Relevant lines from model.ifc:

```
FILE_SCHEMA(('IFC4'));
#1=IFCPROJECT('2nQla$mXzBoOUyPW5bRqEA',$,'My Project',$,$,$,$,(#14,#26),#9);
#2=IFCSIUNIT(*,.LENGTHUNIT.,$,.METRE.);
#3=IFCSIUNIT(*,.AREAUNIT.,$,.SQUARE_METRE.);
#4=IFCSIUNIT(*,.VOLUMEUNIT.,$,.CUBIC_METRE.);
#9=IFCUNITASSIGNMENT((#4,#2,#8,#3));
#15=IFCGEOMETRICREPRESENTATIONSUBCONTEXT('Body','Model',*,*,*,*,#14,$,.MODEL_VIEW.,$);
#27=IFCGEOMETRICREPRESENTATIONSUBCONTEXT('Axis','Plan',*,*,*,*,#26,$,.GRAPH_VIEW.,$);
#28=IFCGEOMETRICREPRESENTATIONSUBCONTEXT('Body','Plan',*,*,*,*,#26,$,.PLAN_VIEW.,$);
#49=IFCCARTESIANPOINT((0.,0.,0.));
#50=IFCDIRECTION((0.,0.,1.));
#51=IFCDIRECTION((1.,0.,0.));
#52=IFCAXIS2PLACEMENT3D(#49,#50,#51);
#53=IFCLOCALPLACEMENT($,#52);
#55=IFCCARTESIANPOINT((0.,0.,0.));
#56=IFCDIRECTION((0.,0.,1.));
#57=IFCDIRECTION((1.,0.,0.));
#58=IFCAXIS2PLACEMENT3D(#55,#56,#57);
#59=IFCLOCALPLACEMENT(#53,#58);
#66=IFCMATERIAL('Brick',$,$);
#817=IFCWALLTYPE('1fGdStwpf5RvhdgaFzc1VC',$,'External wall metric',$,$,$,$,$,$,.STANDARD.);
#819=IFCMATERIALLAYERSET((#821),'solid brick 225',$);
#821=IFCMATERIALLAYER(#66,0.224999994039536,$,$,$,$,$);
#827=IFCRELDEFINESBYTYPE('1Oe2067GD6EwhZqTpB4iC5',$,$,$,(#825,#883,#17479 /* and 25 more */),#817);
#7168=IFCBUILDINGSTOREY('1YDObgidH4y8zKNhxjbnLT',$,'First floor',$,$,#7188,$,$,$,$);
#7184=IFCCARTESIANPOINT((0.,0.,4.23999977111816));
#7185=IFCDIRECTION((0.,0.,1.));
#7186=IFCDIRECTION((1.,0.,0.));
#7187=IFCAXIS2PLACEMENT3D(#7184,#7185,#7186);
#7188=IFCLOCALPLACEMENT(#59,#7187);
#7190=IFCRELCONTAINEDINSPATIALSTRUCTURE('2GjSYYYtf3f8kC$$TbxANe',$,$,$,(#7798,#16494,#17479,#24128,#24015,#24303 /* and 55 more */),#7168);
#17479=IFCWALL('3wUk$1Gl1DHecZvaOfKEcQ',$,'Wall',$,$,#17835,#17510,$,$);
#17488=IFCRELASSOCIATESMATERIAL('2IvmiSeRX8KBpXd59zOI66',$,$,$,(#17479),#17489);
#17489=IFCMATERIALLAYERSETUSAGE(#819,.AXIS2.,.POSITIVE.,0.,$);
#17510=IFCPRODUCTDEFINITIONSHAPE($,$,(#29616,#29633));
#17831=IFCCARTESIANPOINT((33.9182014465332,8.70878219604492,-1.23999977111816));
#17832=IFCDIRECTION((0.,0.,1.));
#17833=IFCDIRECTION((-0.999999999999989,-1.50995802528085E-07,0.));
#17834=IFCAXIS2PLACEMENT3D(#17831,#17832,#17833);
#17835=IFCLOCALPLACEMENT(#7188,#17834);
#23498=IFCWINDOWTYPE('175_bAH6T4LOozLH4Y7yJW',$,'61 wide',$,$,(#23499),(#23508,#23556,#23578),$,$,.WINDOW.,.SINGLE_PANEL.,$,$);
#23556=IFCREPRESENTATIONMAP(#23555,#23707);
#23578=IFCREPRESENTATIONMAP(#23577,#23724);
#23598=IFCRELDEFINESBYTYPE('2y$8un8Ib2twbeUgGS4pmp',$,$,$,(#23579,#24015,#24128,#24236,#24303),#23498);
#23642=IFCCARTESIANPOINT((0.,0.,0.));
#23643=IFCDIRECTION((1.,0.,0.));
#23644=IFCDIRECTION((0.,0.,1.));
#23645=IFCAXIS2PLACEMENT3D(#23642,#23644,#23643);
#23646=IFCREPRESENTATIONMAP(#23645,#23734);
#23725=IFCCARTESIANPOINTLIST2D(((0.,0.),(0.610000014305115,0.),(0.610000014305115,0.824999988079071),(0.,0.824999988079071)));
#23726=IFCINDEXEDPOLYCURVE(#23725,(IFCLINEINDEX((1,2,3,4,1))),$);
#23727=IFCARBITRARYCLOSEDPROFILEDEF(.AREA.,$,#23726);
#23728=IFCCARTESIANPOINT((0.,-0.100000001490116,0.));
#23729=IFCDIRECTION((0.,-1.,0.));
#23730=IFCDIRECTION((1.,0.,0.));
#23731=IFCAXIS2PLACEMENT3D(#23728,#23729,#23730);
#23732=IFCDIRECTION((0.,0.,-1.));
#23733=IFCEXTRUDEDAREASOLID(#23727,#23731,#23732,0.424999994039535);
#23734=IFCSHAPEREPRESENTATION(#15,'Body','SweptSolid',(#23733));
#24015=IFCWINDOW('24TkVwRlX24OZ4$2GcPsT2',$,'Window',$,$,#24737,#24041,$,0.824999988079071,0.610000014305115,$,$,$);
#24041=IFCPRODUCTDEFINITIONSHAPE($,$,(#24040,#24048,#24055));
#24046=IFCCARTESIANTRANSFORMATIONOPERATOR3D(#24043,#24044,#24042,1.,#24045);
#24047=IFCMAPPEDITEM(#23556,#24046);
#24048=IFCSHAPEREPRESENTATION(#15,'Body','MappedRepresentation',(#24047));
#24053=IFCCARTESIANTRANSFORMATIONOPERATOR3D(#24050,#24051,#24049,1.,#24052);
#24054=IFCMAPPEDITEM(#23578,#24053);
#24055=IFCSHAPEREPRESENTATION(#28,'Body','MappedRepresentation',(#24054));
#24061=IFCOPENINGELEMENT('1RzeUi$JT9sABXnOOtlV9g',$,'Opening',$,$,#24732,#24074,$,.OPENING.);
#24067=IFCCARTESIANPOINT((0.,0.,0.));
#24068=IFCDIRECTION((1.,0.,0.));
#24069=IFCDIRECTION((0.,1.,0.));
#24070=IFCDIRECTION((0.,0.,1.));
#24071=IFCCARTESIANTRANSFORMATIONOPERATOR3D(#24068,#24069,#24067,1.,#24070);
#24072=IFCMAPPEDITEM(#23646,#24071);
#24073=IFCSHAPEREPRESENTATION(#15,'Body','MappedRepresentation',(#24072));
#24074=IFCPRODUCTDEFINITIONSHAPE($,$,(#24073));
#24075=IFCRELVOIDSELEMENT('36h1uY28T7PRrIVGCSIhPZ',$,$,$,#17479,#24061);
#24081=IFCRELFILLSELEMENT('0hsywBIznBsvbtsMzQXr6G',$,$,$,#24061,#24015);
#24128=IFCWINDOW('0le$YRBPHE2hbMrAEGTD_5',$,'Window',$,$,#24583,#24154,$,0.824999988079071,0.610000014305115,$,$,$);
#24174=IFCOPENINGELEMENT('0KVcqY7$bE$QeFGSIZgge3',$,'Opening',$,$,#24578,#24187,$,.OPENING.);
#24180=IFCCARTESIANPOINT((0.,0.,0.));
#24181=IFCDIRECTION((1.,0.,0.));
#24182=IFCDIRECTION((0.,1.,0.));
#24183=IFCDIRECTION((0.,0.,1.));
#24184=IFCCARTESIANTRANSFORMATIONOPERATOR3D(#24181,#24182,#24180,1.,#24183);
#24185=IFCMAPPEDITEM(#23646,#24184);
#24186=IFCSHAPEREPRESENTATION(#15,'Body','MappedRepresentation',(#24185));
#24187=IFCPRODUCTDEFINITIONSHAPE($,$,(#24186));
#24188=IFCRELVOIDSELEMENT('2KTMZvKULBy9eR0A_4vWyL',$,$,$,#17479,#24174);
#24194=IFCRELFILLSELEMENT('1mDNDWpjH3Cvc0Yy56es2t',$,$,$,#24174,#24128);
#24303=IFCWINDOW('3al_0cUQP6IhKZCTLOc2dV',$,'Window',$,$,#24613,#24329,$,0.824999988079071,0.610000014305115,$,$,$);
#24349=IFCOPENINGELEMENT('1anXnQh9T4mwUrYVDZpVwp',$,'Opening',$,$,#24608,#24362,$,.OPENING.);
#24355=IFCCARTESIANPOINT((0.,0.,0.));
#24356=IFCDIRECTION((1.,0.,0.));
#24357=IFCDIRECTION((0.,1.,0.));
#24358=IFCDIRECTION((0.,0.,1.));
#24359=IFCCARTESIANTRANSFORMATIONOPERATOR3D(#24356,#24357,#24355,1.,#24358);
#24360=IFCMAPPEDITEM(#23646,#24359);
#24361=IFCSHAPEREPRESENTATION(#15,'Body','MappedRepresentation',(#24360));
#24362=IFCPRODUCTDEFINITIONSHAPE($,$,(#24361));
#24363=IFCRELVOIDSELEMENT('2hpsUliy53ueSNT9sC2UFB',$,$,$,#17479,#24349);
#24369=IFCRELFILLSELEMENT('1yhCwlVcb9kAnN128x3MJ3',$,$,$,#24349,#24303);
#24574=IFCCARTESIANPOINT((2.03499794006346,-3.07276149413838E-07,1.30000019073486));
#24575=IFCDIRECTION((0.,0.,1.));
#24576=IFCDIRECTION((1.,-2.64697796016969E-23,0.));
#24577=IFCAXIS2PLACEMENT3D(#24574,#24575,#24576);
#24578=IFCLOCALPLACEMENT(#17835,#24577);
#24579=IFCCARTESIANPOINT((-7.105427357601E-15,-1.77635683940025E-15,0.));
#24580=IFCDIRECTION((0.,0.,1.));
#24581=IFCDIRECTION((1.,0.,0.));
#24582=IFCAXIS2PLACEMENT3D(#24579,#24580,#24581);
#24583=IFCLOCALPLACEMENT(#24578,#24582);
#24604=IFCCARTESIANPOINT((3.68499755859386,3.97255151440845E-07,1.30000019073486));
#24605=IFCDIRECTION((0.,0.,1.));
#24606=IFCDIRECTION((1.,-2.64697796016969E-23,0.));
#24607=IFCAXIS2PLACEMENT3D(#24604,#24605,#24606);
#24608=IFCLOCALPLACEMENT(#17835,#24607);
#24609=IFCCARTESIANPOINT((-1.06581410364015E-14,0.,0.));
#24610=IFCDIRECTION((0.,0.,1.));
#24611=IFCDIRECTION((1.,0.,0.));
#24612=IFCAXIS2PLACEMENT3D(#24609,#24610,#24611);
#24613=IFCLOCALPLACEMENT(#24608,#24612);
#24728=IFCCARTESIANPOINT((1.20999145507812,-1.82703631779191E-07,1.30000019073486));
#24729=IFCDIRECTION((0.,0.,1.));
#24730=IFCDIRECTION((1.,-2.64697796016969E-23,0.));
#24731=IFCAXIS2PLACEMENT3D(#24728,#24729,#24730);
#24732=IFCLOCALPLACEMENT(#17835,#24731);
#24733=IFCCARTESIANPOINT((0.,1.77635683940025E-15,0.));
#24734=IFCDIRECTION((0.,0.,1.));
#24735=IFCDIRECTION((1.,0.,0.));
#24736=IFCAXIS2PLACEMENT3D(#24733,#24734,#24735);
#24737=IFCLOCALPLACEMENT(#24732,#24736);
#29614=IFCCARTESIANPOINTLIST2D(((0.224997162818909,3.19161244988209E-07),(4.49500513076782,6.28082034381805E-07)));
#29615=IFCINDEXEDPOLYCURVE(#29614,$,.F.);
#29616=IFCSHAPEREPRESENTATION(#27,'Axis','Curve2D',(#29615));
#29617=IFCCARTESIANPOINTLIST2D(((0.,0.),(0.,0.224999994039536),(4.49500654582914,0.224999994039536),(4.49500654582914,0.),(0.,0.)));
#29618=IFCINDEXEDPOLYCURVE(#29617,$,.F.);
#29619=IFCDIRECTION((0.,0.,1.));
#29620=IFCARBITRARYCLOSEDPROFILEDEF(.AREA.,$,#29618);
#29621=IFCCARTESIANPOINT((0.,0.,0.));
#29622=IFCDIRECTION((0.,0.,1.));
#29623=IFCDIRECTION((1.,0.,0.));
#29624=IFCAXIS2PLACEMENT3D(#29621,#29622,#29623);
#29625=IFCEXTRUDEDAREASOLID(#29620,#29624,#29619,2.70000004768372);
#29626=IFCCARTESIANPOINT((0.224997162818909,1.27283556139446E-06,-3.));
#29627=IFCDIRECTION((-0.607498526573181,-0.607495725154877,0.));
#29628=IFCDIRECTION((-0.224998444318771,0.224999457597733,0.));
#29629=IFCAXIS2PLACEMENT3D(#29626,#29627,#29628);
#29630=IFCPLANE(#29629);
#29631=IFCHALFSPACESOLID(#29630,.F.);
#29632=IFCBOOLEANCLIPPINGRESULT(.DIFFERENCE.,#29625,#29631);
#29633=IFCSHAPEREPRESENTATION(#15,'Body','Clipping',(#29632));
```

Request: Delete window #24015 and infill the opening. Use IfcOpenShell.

```python
import ifcopenshell
import ifcopenshell.api.feature
import ifcopenshell.api.root
import ifcopenshell.geom
import ifcopenshell.util.shape

model = ifcopenshell.open("model.ifc")
settings = ifcopenshell.geom.settings()


def volume(element):
    """Net volume in cubic metres, openings subtracted."""
    shape = ifcopenshell.geom.create_shape(settings, element)
    return ifcopenshell.util.shape.get_volume(shape.geometry)


window = model.by_id(24015)
opening = window.FillsVoids[0].RelatingOpeningElement
wall = opening.VoidsElements[0].RelatingBuildingElement
before = volume(wall)

ifcopenshell.api.root.remove_product(model, product=window)
ifcopenshell.api.feature.remove_feature(model, feature=opening)

after = volume(wall)

print(f"wall volume {before:.3f} -> {after:.3f} m3")

model.write("model_updated.ifc")
```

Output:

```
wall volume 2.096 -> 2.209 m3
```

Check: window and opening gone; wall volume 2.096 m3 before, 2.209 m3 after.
